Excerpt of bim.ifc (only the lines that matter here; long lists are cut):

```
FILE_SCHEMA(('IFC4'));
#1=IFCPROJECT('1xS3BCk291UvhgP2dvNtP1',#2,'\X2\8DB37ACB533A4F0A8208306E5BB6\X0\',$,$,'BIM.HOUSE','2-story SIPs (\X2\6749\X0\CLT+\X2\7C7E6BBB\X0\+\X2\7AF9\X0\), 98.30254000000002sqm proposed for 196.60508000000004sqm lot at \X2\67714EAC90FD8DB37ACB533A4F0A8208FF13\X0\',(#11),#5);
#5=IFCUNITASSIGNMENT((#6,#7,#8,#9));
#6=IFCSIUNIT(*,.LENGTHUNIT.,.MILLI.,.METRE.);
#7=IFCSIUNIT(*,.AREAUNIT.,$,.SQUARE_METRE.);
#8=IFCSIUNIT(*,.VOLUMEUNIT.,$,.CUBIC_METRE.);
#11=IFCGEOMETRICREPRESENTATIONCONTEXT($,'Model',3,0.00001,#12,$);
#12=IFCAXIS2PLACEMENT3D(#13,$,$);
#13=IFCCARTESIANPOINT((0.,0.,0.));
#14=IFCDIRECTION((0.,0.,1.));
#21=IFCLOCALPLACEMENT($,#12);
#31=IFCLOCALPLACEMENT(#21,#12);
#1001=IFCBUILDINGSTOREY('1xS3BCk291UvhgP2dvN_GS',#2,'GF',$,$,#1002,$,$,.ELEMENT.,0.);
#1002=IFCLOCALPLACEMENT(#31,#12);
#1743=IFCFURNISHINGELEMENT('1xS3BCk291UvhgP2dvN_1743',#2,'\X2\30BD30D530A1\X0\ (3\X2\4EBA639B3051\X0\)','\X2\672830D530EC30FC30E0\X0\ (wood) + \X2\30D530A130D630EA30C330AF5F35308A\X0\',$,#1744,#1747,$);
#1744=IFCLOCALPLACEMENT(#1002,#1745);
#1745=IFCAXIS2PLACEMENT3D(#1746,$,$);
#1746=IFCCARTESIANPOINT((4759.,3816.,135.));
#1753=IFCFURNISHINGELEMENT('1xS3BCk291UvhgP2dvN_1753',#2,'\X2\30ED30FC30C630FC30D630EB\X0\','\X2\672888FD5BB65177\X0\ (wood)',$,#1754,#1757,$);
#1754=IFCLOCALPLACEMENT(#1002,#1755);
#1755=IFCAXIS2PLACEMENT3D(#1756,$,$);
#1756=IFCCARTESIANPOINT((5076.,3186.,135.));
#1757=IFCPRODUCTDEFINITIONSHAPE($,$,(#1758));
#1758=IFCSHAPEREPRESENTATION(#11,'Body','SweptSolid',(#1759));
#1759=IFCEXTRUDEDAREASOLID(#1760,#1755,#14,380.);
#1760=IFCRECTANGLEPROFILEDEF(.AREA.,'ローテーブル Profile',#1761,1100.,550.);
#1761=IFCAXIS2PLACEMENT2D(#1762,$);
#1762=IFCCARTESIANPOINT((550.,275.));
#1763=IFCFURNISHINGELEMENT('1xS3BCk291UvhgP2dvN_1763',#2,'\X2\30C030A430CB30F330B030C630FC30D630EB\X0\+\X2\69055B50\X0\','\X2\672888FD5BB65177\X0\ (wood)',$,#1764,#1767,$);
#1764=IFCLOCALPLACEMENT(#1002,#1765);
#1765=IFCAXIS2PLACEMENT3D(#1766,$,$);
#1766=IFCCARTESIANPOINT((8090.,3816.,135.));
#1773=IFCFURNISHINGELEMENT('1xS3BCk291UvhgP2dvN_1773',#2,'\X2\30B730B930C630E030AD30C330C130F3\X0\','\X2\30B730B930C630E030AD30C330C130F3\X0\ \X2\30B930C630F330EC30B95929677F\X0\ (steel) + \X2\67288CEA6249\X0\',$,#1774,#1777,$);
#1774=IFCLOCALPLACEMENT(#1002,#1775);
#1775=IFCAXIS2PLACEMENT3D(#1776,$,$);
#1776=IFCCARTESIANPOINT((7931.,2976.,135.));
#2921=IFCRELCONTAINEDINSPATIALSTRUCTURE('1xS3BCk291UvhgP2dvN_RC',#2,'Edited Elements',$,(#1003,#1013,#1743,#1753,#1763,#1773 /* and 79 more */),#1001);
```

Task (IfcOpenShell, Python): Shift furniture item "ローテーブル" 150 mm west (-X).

```python
import ifcopenshell
import ifcopenshell.api.geometry
import ifcopenshell.util.placement

model = ifcopenshell.open("bim.ifc")

item = model.by_id(1753)
matrix = ifcopenshell.util.placement.get_local_placement(item.ObjectPlacement)
matrix[0, 3] -= 150.0
ifcopenshell.api.geometry.edit_object_placement(model, product=item, matrix=matrix, is_si=False)

print(ifcopenshell.util.placement.get_local_placement(item.ObjectPlacement).round(3) + 0.0)

model.write("bim_v2.ifc")
```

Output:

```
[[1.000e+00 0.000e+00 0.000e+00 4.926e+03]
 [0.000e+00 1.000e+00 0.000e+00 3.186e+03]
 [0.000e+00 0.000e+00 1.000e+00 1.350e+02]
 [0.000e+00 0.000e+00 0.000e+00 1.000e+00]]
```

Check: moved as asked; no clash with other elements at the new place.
